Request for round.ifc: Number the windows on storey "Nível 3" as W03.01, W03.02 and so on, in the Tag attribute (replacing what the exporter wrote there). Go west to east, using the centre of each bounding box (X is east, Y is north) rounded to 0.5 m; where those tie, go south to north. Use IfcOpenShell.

First a look at what the model holds.

```python
import ifcopenshell
import ifcopenshell.util.element
import ifcopenshell.util.placement

model = ifcopenshell.open("round.ifc")
print(model.schema)
storey = next(s for s in model.by_type("IfcBuildingStorey") if s.Name == "Nível 3")
windows = [e for e in ifcopenshell.util.element.get_decomposition(storey) if e.is_a("IfcWindow")]
for e in sorted(windows, key=lambda e: e.id()):
    origin = ifcopenshell.util.placement.get_local_placement(e.ObjectPlacement)[:3, 3]
    print(e.id(), e.Tag, e.Name, origin.round(2) + 0.0, sep=" | ")
```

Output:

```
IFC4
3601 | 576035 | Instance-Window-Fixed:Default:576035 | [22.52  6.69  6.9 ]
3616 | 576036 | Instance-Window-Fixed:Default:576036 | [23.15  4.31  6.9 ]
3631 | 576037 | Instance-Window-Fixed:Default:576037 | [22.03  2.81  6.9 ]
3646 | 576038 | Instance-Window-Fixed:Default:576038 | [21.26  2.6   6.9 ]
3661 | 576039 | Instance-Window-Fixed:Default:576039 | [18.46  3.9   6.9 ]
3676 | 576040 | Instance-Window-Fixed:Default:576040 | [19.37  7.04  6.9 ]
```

```python
import ifcopenshell
import ifcopenshell.geom
import ifcopenshell.util.element
import ifcopenshell.util.shape

model = ifcopenshell.open("round.ifc")
settings = ifcopenshell.geom.settings()
settings.set("use-world-coords", True)


def centre(element):
    shape = ifcopenshell.geom.create_shape(settings, element)
    return ifcopenshell.util.shape.get_bbox_centroid(shape.geometry)


storey = next(s for s in model.by_type("IfcBuildingStorey") if s.Name == "Nível 3")
windows = [e for e in ifcopenshell.util.element.get_decomposition(storey) if e.is_a("IfcWindow")]

# Insertion points can sit at a corner or the storey origin, so sort by the geometry (in metres).
centres = {e: centre(e) for e in windows}
windows.sort(key=lambda e: (round(centres[e][0] / 0.5), centres[e][1]))

for i, e in enumerate(windows, start=1):
    number = f"W03.{i:02d}"
    e.Tag = number
    print(e.id(), number)

model.write("round_v2.ifc")
```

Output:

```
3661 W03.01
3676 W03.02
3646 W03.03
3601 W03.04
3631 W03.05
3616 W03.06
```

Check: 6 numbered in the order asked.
